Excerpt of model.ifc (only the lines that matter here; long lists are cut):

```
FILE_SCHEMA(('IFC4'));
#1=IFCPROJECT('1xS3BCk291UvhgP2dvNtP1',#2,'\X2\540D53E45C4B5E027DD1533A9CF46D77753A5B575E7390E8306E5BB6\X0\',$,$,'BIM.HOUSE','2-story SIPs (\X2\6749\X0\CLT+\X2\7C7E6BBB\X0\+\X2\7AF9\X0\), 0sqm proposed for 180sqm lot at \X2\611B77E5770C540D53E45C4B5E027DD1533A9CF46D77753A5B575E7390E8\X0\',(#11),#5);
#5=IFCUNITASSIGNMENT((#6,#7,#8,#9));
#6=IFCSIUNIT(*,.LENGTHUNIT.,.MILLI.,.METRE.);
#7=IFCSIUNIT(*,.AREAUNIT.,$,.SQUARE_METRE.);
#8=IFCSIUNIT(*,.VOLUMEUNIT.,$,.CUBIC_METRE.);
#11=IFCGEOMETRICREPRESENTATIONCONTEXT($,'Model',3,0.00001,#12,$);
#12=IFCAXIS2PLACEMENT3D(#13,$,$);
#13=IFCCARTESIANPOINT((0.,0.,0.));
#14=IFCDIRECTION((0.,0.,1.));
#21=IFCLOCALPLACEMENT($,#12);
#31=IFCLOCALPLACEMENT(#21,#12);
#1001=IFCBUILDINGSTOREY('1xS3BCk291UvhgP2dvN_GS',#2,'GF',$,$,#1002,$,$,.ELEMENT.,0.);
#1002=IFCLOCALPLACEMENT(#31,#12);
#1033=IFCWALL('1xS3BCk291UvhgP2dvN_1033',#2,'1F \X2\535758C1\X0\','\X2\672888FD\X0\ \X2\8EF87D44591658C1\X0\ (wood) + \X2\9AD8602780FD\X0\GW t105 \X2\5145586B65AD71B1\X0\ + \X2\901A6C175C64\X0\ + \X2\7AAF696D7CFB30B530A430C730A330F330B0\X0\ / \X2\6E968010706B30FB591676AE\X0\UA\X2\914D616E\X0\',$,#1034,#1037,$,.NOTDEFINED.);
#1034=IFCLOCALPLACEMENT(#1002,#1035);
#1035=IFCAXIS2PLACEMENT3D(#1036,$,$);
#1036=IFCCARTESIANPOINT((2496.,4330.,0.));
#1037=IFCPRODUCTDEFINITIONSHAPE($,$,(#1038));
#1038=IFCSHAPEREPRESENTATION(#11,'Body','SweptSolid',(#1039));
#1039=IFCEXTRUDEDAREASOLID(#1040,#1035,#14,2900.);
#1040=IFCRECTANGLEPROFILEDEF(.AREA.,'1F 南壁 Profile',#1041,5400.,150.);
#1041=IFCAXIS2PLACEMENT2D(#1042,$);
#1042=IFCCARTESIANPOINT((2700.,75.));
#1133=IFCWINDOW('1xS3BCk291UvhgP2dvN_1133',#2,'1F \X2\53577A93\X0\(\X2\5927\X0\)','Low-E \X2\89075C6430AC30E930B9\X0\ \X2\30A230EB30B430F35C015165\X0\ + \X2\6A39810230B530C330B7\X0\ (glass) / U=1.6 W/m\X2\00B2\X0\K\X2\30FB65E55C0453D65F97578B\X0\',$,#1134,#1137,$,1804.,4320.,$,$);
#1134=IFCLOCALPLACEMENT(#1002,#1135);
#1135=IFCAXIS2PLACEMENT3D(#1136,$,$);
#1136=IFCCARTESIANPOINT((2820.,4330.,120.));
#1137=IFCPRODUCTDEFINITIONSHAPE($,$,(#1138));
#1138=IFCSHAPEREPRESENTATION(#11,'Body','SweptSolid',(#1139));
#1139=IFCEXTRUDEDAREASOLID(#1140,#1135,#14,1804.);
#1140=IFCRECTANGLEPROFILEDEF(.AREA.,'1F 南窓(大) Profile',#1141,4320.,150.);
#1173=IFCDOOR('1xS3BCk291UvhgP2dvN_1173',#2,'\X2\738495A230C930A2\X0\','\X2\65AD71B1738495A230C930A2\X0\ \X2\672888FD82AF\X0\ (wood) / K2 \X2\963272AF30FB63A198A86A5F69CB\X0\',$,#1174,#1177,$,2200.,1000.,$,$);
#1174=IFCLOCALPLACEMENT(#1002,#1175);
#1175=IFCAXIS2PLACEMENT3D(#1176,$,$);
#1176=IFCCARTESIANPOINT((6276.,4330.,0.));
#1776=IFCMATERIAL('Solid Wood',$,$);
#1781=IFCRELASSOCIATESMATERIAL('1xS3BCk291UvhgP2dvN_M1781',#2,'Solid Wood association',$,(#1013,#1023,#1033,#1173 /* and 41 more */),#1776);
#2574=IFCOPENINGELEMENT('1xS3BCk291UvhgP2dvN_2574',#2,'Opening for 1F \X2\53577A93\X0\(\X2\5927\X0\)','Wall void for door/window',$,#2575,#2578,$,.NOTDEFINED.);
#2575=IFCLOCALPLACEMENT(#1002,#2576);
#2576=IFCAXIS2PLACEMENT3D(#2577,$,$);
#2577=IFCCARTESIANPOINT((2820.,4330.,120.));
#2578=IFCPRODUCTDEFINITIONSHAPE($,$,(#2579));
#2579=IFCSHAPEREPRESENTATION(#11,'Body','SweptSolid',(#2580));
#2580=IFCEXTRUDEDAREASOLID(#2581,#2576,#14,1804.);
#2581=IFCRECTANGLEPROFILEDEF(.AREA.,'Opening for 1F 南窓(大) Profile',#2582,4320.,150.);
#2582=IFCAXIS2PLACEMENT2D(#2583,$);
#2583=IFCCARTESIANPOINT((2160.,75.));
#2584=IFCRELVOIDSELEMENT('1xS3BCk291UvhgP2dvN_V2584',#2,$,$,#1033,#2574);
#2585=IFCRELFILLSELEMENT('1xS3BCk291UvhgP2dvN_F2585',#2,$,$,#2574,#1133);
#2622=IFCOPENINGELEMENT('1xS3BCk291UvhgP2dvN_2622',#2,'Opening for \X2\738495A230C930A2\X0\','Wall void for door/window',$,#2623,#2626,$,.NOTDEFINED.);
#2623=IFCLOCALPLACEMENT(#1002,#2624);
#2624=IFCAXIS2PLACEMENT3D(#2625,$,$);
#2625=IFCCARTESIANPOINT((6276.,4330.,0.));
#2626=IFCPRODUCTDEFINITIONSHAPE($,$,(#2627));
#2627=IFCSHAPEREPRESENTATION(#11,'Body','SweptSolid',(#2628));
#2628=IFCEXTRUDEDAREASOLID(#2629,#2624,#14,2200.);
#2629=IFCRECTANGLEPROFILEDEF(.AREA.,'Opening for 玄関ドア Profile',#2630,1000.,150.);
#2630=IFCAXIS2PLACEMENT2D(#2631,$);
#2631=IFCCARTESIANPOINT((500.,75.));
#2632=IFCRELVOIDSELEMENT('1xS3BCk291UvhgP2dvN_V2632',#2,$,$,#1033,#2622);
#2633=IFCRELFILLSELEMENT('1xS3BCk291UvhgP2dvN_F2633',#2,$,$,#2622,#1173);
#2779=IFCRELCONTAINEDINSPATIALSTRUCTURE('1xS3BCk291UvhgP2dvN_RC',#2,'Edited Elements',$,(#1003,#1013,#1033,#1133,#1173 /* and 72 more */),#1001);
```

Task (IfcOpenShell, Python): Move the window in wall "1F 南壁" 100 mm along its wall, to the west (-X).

```python
import ifcopenshell
import ifcopenshell.api.geometry
import ifcopenshell.util.placement
import ifcopenshell.util.unit

model = ifcopenshell.open("model.ifc")
unit_scale = ifcopenshell.util.unit.calculate_unit_scale(model)

window = model.by_guid("1xS3BCk291UvhgP2dvN_1133")
opening = window.FillsVoids[0].RelatingOpeningElement
wall = opening.VoidsElements[0].RelatingBuildingElement

wall_matrix = ifcopenshell.util.placement.get_local_placement(wall.ObjectPlacement)
shift = wall_matrix[:3, 0] * -0.1 / unit_scale
before = ifcopenshell.util.placement.get_local_placement(window.ObjectPlacement)[:3, 3].copy()

# The window is not placed relative to its opening, so move both.
for product in (opening, window):
    matrix = ifcopenshell.util.placement.get_local_placement(product.ObjectPlacement)
    matrix[:3, 3] += shift
    ifcopenshell.api.geometry.edit_object_placement(model, product=product, matrix=matrix, is_si=False)

after = ifcopenshell.util.placement.get_local_placement(window.ObjectPlacement)[:3, 3]
print("window moved by", (after - before).round(3) + 0.0)

model.write("model_updated.ifc")
```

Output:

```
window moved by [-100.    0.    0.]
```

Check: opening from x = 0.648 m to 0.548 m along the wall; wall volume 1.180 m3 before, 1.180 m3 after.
